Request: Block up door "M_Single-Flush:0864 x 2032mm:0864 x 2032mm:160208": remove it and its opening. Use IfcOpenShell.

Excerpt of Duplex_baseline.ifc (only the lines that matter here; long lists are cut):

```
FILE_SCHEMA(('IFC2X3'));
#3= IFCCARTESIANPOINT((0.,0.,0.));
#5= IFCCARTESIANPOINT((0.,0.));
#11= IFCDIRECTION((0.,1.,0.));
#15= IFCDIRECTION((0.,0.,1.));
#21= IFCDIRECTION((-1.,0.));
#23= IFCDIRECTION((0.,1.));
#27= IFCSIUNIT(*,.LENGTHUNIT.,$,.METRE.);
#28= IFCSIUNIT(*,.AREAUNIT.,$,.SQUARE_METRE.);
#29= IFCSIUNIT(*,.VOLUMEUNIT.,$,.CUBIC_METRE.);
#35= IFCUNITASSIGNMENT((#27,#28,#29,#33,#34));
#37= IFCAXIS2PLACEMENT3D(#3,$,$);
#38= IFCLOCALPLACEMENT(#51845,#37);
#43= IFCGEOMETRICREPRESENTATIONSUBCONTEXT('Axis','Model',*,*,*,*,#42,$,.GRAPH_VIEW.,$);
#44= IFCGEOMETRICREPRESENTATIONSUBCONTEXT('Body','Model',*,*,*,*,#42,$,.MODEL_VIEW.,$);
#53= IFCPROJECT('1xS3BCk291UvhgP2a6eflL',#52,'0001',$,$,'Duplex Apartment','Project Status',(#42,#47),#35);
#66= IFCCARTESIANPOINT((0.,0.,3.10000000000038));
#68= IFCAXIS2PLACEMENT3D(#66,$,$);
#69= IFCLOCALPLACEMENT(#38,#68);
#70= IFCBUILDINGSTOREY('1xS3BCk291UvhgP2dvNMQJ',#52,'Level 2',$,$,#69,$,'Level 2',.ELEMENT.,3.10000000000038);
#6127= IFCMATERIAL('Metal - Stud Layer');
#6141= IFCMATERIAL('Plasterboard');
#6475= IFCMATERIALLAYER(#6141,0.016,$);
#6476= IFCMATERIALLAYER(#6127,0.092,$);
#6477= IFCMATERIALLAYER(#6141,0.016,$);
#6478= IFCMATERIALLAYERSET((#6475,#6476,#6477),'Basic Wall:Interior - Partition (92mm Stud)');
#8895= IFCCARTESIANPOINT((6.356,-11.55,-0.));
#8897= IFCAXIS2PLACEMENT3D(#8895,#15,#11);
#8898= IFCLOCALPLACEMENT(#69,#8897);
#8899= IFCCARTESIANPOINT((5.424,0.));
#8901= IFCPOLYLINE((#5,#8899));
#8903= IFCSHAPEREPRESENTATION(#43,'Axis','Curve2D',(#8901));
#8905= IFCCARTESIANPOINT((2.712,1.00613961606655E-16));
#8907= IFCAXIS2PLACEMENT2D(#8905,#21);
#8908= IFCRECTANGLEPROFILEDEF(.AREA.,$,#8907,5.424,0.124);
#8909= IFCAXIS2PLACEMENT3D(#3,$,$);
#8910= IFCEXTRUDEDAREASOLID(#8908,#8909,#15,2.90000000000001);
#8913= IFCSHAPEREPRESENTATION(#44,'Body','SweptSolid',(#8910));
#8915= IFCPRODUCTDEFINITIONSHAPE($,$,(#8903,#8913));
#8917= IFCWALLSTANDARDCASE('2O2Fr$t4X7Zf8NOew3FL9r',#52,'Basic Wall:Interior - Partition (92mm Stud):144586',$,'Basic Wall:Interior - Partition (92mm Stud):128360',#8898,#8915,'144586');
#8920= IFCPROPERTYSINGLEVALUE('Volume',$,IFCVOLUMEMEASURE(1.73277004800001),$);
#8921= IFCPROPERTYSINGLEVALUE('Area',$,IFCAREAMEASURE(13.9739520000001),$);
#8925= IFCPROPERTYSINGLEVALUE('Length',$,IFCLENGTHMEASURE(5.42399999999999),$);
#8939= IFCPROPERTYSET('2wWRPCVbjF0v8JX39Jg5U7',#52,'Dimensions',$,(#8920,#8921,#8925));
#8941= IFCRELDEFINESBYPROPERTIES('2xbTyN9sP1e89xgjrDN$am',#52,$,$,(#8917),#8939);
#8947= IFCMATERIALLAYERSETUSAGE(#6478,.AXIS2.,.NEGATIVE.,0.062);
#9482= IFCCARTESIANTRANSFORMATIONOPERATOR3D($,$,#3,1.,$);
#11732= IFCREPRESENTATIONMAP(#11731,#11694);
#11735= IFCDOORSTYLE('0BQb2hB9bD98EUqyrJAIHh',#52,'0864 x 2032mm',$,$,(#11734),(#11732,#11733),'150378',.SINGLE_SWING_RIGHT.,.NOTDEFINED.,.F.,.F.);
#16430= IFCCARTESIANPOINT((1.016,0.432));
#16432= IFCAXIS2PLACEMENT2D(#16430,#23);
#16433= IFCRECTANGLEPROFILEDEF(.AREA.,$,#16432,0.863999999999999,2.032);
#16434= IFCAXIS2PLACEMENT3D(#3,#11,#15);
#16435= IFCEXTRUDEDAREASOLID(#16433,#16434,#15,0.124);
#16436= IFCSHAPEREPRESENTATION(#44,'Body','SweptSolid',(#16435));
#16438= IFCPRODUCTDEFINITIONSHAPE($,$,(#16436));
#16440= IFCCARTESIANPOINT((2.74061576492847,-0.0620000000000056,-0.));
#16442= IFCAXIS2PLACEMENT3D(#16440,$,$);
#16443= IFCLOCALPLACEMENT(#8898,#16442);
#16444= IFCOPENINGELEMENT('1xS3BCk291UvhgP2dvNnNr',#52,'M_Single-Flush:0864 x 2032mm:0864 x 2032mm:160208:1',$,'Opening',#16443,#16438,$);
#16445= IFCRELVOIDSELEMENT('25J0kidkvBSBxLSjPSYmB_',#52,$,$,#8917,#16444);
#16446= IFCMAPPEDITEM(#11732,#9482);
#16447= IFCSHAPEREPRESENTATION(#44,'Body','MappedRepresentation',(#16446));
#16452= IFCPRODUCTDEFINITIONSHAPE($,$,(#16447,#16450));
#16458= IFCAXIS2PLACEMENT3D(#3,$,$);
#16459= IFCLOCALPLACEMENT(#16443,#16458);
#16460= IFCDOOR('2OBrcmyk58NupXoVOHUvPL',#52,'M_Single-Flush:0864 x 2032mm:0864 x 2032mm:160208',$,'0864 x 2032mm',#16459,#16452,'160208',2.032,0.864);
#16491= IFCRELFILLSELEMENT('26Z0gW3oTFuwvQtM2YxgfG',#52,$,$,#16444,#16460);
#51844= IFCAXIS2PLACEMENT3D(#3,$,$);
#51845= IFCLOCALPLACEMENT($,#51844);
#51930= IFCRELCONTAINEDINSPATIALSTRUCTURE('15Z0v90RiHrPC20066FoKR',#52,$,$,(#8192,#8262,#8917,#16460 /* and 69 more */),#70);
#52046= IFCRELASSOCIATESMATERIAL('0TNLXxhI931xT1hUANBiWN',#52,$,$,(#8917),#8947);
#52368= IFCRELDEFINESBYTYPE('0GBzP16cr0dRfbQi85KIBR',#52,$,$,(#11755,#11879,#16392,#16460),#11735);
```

```python
import ifcopenshell
import ifcopenshell.api.feature
import ifcopenshell.api.pset
import ifcopenshell.api.root
import ifcopenshell.geom
import ifcopenshell.util.element
import ifcopenshell.util.shape
import ifcopenshell.util.unit

model = ifcopenshell.open("Duplex_baseline.ifc")
area_scale = ifcopenshell.util.unit.calculate_unit_scale(model, "AREAUNIT")
volume_scale = ifcopenshell.util.unit.calculate_unit_scale(model, "VOLUMEUNIT")
settings = ifcopenshell.geom.settings()


def volume(element):
    """Net volume in cubic metres, openings subtracted."""
    shape = ifcopenshell.geom.create_shape(settings, element)
    return ifcopenshell.util.shape.get_volume(shape.geometry)


door = model.by_guid("2OBrcmyk58NupXoVOHUvPL")
opening = door.FillsVoids[0].RelatingOpeningElement
wall = opening.VoidsElements[0].RelatingBuildingElement
before = volume(wall)

ifcopenshell.api.root.remove_product(model, product=door)
ifcopenshell.api.feature.remove_feature(model, feature=opening)

after = volume(wall)
thickness = 0.124  # wall thickness in metres

# Update the wall's stored quantities.
pset = model.by_id(ifcopenshell.util.element.get_pset(wall, "Dimensions", should_inherit=False)["id"])
ifcopenshell.api.pset.edit_pset(model, pset=pset, properties={
    "Volume": model.create_entity("IfcVolumeMeasure", after / volume_scale),
    "Area": model.create_entity("IfcAreaMeasure", after / thickness / area_scale),
})

print(f"wall volume {before:.3f} -> {after:.3f} m3")

model.write("Duplex_baseline_edited.ifc")
```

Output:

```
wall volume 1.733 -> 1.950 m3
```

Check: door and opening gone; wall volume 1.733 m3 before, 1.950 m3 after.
